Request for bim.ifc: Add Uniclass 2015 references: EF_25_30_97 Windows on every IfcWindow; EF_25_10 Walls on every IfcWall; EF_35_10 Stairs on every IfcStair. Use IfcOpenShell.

First a look at what the model holds.

```python
import ifcopenshell

model = ifcopenshell.open("bim.ifc")
print(model.schema)
print("classifications:", [c.Name for c in model.by_type("IfcClassification")])
for ifc_class in ("IfcDoor", "IfcRoof", "IfcStair", "IfcWall", "IfcWindow"):
    print(ifc_class, len(model.by_type(ifc_class)))
```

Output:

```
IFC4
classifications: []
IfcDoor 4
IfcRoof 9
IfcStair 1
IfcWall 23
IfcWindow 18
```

```python
import ifcopenshell
import ifcopenshell.api.classification

model = ifcopenshell.open("bim.ifc")

system = ifcopenshell.api.classification.add_classification(model, classification="Uniclass 2015")

codes = {
    "IfcWindow": ("EF_25_30_97", "Windows"),
    "IfcWall": ("EF_25_10", "Walls"),
    "IfcStair": ("EF_35_10", "Stairs"),
}
for ifc_class, (code, name) in codes.items():
    products = model.by_type(ifc_class)
    ifcopenshell.api.classification.add_reference(
        model, products=products, classification=system, identification=code, name=name
    )
    print(code, len(products))

model.write("bim_v2.ifc")
```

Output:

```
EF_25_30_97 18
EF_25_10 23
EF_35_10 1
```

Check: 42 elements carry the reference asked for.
